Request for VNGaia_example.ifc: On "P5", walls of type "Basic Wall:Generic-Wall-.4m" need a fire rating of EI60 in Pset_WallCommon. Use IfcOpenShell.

First a look at what the model holds.

```python
import ifcopenshell
import ifcopenshell.util.element

model = ifcopenshell.open("VNGaia_example.ifc")
print(model.schema)
storey = next(s for s in model.by_type("IfcBuildingStorey") if s.Name == "P5")
walls = [e for e in ifcopenshell.util.element.get_decomposition(storey) if e.is_a("IfcWall")]
seen = {}
for e in walls:
    element_type = ifcopenshell.util.element.get_type(e)
    key = (element_type.Name if element_type != e and element_type else None, ifcopenshell.util.element.get_pset(e, "Pset_WallCommon", "FireRating"))
    seen[key] = seen.get(key, 0) + 1
for (name, value), count in sorted(seen.items(), key=str):
    print(count, "x", name, "|", value)
```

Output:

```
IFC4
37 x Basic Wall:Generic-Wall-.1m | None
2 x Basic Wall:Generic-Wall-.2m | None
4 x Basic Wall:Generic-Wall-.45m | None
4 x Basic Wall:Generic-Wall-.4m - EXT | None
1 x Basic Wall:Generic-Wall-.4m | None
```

```python
import ifcopenshell
import ifcopenshell.api.pset
import ifcopenshell.util.element

model = ifcopenshell.open("VNGaia_example.ifc")

storey = next(s for s in model.by_type("IfcBuildingStorey") if s.Name == "P5")
walls = [e for e in ifcopenshell.util.element.get_decomposition(storey) if e.is_a("IfcWall")]

count = 0
for e in walls:
    element_type = ifcopenshell.util.element.get_type(e)
    if element_type in (None, e) or element_type.Name != "Basic Wall:Generic-Wall-.4m":
        continue
    # add_pset returns the element's existing set when there is one.
    pset = ifcopenshell.api.pset.add_pset(model, product=e, name="Pset_WallCommon")
    ifcopenshell.api.pset.edit_pset(model, pset=pset, properties={"FireRating": "EI60"})
    count += 1

print(count, "walls updated")

model.write("VNGaia_example-out.ifc")
```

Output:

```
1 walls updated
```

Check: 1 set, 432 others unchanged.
